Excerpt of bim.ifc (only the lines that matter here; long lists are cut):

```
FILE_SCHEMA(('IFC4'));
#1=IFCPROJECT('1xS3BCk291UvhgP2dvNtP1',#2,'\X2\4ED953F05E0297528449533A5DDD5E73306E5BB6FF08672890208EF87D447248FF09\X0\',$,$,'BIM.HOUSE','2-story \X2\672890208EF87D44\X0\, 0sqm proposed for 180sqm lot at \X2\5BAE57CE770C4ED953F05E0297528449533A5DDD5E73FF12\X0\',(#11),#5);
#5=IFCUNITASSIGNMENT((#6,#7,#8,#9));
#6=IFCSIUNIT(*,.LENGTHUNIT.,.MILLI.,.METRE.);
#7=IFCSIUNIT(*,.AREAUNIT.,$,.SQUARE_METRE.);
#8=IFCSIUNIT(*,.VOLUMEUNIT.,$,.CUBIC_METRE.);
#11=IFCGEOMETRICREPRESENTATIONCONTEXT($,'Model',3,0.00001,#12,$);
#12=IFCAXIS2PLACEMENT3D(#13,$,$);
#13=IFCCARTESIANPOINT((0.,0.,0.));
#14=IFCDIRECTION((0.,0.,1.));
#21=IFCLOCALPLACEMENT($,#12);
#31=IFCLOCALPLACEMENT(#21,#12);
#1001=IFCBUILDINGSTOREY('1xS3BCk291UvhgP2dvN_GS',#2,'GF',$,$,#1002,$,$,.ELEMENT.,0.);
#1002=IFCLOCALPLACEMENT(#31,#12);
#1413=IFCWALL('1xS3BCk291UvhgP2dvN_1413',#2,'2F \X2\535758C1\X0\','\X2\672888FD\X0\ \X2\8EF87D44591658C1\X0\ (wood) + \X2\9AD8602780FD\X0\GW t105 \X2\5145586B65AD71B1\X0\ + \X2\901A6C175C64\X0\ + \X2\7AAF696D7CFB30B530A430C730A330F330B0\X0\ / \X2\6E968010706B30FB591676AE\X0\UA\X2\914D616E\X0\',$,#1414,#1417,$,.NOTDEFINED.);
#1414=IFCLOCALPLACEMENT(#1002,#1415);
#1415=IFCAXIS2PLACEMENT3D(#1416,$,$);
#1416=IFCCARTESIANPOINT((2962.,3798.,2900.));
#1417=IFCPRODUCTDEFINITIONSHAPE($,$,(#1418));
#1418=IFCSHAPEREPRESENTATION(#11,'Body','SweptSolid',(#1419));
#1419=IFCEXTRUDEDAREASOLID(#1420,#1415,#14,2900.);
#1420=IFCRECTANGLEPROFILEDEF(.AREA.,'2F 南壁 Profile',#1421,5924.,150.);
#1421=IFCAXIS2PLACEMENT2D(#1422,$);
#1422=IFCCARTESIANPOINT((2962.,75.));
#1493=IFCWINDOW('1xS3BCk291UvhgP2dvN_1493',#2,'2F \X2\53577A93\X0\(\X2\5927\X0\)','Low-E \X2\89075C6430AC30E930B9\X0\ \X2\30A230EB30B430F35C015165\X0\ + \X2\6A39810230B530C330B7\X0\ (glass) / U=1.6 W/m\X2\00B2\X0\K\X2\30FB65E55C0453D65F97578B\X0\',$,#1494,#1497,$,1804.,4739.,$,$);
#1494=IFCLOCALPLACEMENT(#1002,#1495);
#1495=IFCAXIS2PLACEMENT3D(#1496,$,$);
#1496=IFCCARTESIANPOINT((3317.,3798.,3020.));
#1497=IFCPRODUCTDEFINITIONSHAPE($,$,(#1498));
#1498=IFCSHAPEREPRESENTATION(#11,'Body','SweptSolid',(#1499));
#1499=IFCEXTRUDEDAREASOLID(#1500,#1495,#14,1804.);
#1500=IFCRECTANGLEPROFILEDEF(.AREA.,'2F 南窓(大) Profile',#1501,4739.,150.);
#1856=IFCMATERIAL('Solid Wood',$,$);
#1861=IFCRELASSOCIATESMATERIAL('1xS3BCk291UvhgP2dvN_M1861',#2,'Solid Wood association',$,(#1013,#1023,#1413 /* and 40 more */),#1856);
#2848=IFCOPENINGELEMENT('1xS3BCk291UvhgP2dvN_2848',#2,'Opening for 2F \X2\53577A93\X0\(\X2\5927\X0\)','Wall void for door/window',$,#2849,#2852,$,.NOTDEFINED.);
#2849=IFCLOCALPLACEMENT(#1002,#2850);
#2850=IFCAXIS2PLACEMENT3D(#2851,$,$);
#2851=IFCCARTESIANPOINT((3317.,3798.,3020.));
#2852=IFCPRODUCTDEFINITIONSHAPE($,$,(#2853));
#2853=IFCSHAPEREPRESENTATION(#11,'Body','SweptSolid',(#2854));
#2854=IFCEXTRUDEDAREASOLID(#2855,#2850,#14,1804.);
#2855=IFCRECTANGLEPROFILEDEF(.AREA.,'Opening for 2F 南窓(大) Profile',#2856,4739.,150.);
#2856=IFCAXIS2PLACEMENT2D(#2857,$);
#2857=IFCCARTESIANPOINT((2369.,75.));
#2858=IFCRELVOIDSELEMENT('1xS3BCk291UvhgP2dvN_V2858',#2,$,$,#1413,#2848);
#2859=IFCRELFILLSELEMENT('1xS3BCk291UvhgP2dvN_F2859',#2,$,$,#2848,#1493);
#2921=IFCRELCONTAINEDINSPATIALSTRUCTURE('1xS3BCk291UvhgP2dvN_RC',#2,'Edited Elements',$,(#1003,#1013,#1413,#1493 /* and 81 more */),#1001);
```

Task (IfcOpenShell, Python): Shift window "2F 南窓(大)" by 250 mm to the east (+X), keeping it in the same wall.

```python
import ifcopenshell
import ifcopenshell.api.geometry
import ifcopenshell.util.placement

model = ifcopenshell.open("bim.ifc")

window = model.by_guid("1xS3BCk291UvhgP2dvN_1493")
opening = window.FillsVoids[0].RelatingOpeningElement
wall = opening.VoidsElements[0].RelatingBuildingElement

wall_matrix = ifcopenshell.util.placement.get_local_placement(wall.ObjectPlacement)
shift = wall_matrix[:3, 0] * 250.0
before = ifcopenshell.util.placement.get_local_placement(window.ObjectPlacement)[:3, 3].copy()

# The window is not placed relative to its opening, so move both.
for product in (opening, window):
    matrix = ifcopenshell.util.placement.get_local_placement(product.ObjectPlacement)
    matrix[:3, 3] += shift
    ifcopenshell.api.geometry.edit_object_placement(model, product=product, matrix=matrix, is_si=False)

after = ifcopenshell.util.placement.get_local_placement(window.ObjectPlacement)[:3, 3]
print("window moved by", (after - before).round(3) + 0.0)

model.write("bim_rev.ifc")
```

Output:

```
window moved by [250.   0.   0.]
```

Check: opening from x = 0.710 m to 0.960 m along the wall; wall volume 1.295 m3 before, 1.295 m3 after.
